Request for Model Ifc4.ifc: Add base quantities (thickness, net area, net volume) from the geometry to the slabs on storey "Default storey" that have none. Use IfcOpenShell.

First a look at what the model holds.

```python
import ifcopenshell
import ifcopenshell.util.element
import ifcopenshell.util.unit

model = ifcopenshell.open("Model Ifc4.ifc")
print(model.schema)
for unit_type in ("LENGTHUNIT", "AREAUNIT", "VOLUMEUNIT"):
    print(unit_type, ifcopenshell.util.unit.calculate_unit_scale(model, unit_type))
storey = next(s for s in model.by_type("IfcBuildingStorey") if s.Name == "Default storey")
slabs = [e for e in ifcopenshell.util.element.get_decomposition(storey) if e.is_a("IfcSlab")]
for e in sorted(slabs, key=lambda e: e.id()):
    print(e.id(), e.is_a(), e.Name, list(ifcopenshell.util.element.get_psets(e, qtos_only=True)), sep=" | ")
```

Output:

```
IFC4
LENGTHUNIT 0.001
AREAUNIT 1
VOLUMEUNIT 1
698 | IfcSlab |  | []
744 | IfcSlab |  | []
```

```python
import ifcopenshell
import ifcopenshell.api.pset
import ifcopenshell.geom
import ifcopenshell.util.element
import ifcopenshell.util.shape
import ifcopenshell.util.unit

model = ifcopenshell.open("Model Ifc4.ifc")
unit_scale = ifcopenshell.util.unit.calculate_unit_scale(model)
area_scale = ifcopenshell.util.unit.calculate_unit_scale(model, "AREAUNIT")
volume_scale = ifcopenshell.util.unit.calculate_unit_scale(model, "VOLUMEUNIT")
settings = ifcopenshell.geom.settings()

storey = next(s for s in model.by_type("IfcBuildingStorey") if s.Name == "Default storey")
slabs = [e for e in ifcopenshell.util.element.get_decomposition(storey) if e.is_a("IfcSlab")]

for e in sorted(slabs, key=lambda e: e.id()):
    if ifcopenshell.util.element.get_psets(e, qtos_only=True, should_inherit=False):
        continue
    # Geometry comes back in metres, in the element's own axes.
    shape = ifcopenshell.geom.create_shape(settings, e)
    values = {
        "Width": ifcopenshell.util.shape.get_z(shape.geometry) / unit_scale,
        "NetArea": ifcopenshell.util.shape.get_footprint_area(shape.geometry) / area_scale,
        "NetVolume": ifcopenshell.util.shape.get_volume(shape.geometry) / volume_scale,
    }
    qto = ifcopenshell.api.pset.add_qto(model, product=e, name="Qto_SlabBaseQuantities")
    ifcopenshell.api.pset.edit_qto(model, qto=qto, properties=values)
    print(e.id(), {k: round(v, 3) for k, v in values.items()})

model.write("Model Ifc4_edited.ifc")
```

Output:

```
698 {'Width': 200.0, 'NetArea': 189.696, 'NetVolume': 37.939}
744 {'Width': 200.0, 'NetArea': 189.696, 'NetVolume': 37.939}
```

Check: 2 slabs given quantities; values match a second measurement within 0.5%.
